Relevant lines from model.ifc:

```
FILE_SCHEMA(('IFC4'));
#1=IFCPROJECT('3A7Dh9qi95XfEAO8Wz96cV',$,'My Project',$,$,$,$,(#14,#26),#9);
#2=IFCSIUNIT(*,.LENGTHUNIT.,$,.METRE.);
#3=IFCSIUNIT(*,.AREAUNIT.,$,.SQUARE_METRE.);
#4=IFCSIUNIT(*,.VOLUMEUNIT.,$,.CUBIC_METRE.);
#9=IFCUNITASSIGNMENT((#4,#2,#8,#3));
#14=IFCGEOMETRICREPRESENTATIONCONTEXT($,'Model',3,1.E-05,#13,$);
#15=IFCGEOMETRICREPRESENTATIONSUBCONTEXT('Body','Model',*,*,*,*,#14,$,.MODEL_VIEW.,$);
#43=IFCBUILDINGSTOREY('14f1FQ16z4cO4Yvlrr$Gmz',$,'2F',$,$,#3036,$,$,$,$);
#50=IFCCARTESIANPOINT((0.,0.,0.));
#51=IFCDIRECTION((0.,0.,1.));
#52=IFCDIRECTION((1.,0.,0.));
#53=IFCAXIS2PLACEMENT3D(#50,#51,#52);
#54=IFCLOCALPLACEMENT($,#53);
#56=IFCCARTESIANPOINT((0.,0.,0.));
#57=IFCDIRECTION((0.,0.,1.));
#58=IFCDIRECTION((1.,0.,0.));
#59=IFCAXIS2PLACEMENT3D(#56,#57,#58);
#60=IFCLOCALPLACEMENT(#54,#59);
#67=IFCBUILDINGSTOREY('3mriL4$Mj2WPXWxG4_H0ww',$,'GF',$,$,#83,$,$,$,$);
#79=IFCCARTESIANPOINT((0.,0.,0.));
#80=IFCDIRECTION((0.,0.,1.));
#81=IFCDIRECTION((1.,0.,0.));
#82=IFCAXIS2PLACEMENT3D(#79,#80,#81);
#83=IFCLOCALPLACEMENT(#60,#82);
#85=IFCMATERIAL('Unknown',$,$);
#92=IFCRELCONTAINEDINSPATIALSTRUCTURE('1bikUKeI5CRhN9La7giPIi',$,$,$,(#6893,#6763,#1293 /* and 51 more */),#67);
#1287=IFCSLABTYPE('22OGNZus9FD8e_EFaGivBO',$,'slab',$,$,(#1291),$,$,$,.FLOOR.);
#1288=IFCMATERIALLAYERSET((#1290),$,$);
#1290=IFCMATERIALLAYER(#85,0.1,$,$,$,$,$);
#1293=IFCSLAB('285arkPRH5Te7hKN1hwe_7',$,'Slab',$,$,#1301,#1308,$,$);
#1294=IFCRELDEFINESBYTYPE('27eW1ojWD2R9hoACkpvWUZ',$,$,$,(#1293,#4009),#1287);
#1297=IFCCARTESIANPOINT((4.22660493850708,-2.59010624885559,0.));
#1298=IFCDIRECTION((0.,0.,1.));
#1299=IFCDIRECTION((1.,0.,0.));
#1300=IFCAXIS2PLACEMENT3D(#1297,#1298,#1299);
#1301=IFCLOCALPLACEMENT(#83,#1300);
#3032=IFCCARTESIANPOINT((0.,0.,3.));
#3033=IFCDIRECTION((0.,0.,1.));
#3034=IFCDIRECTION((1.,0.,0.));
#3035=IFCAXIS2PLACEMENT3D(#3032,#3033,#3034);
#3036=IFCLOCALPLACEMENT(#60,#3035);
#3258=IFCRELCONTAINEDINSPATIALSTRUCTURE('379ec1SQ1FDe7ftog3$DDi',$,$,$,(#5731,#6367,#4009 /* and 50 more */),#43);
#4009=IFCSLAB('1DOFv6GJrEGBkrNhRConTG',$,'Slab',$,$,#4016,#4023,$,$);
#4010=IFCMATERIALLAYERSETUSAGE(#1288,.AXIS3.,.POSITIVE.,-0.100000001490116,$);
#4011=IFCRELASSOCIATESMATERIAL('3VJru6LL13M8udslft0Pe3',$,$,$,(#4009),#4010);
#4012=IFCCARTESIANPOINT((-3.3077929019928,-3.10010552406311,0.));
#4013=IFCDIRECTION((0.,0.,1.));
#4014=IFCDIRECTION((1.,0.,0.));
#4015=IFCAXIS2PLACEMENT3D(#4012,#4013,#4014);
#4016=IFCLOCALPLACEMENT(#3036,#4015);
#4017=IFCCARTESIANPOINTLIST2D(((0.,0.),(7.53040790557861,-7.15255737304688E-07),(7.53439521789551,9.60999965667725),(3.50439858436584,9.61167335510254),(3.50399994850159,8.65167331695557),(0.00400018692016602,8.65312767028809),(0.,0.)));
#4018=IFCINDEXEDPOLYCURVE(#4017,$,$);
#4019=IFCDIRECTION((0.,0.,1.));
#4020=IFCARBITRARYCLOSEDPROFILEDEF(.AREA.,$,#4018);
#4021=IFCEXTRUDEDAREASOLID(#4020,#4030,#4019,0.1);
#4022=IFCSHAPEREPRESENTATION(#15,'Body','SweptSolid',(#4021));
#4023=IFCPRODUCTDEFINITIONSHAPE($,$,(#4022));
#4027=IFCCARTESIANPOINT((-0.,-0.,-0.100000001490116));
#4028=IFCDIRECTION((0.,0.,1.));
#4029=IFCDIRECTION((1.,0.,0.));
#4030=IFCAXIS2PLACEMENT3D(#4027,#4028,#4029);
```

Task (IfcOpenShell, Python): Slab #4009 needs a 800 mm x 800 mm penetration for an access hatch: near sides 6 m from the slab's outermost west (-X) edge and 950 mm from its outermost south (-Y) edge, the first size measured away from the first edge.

```python
import numpy as np
import ifcopenshell
import ifcopenshell.api.feature
import ifcopenshell.api.geometry
import ifcopenshell.api.root
import ifcopenshell.geom
import ifcopenshell.util.placement
import ifcopenshell.util.representation
import ifcopenshell.util.shape
import ifcopenshell.util.unit

model = ifcopenshell.open("model.ifc")
unit_scale = ifcopenshell.util.unit.calculate_unit_scale(model)
settings = ifcopenshell.geom.settings()


def volume(element):
    """Net volume in cubic metres, openings subtracted."""
    shape = ifcopenshell.geom.create_shape(settings, element)
    return ifcopenshell.util.shape.get_volume(shape.geometry)


slab = model.by_guid("1DOFv6GJrEGBkrNhRConTG")
before = volume(slab)

# Extent in the slab's own axes, in metres. The edges named are its -X and -Y sides.
slab_shape = ifcopenshell.geom.create_shape(settings, slab)
vertices = ifcopenshell.util.shape.get_vertices(slab_shape.geometry)
x_min, y_min, bottom = vertices.min(axis=0)
top = vertices[:, 2].max()

opening = ifcopenshell.api.root.create_entity(model, ifc_class="IfcOpeningElement", name="Access hatch opening", predefined_type="OPENING")
context = ifcopenshell.util.representation.get_context(model, "Model", "Body", "MODEL_VIEW")
width, depth = 0.8, 0.8
outline = [(0.0, 0.0), (width, 0.0), (width, depth), (0.0, depth), (0.0, 0.0)]
# Overshoot both faces by 50 mm so the cut is clean.
shape = ifcopenshell.api.geometry.add_slab_representation(
    model, context=context, depth=top - bottom + 0.1, polyline=outline
)
ifcopenshell.api.geometry.assign_representation(model, product=opening, representation=shape)

matrix = ifcopenshell.util.placement.get_local_placement(slab.ObjectPlacement)
matrix[:, 3] = matrix @ np.append(np.array([x_min + 6, y_min + 0.95, bottom - 0.05]) / unit_scale, 1.0)
ifcopenshell.api.geometry.edit_object_placement(model, product=opening, matrix=matrix, is_si=False)
ifcopenshell.api.feature.add_feature(model, feature=opening, element=slab)

after = volume(slab)

print(f"slab volume {before:.3f} -> {after:.3f} m3")

model.write("model_updated.ifc")
```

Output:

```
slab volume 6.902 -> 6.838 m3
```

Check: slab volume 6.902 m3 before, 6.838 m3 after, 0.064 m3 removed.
